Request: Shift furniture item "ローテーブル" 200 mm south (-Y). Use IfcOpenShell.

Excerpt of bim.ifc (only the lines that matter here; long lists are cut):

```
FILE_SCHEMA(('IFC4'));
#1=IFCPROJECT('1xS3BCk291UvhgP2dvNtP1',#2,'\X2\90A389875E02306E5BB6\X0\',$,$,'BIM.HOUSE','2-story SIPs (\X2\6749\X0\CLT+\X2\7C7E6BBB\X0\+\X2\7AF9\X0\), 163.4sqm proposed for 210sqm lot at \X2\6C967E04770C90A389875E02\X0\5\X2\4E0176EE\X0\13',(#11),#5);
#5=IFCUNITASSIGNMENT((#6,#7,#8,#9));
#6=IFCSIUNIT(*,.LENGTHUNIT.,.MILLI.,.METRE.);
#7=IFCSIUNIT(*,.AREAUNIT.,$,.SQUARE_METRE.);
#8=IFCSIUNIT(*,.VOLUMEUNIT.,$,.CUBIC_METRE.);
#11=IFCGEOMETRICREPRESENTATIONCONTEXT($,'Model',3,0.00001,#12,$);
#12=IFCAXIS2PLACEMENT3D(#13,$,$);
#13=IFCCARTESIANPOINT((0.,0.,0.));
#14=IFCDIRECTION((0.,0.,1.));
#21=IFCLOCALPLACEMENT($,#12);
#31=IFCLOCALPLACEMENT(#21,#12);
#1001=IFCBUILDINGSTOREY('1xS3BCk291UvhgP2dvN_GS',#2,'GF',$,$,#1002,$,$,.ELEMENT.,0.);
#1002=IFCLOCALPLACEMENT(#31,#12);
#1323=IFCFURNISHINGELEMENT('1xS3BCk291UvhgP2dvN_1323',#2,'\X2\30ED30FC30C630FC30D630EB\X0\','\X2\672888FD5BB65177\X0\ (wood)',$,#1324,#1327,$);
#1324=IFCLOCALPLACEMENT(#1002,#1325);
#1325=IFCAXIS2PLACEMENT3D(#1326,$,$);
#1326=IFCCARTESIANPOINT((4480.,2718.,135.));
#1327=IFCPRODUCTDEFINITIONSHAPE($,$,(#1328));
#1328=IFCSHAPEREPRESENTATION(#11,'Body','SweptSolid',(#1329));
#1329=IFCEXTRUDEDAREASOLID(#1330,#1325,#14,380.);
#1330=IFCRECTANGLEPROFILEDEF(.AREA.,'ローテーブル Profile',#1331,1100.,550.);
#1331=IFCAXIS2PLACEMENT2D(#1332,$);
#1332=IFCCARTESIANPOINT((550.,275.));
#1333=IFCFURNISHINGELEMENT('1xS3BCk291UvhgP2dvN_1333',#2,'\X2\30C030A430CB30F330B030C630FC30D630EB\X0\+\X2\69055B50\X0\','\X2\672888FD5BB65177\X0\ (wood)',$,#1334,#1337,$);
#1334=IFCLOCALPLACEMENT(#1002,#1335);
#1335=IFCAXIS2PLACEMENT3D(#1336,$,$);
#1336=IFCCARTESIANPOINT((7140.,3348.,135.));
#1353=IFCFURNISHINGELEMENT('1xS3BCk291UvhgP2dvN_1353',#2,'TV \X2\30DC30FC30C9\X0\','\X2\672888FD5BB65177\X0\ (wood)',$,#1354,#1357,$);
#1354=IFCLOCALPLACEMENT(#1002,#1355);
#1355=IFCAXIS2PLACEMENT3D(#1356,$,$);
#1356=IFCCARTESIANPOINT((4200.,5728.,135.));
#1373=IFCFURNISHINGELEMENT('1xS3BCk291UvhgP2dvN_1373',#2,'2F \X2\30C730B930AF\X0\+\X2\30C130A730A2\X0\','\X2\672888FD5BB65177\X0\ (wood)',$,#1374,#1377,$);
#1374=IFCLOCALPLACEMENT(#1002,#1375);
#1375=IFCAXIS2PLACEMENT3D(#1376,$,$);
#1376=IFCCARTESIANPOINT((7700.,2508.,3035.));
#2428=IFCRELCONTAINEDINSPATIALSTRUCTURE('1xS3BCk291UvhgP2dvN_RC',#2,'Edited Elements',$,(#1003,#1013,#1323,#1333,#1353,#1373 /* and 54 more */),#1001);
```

```python
import ifcopenshell
import ifcopenshell.api.geometry
import ifcopenshell.util.placement
import ifcopenshell.util.unit

model = ifcopenshell.open("bim.ifc")
unit_scale = ifcopenshell.util.unit.calculate_unit_scale(model)

item = model.by_id(1323)
matrix = ifcopenshell.util.placement.get_local_placement(item.ObjectPlacement)
matrix[1, 3] -= 0.2 / unit_scale
ifcopenshell.api.geometry.edit_object_placement(model, product=item, matrix=matrix, is_si=False)

print(ifcopenshell.util.placement.get_local_placement(item.ObjectPlacement).round(3) + 0.0)

model.write("bim-out.ifc")
```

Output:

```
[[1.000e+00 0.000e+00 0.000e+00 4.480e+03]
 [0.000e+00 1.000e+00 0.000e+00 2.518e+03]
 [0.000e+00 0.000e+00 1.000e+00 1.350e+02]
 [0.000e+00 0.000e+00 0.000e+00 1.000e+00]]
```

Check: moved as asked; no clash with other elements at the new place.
